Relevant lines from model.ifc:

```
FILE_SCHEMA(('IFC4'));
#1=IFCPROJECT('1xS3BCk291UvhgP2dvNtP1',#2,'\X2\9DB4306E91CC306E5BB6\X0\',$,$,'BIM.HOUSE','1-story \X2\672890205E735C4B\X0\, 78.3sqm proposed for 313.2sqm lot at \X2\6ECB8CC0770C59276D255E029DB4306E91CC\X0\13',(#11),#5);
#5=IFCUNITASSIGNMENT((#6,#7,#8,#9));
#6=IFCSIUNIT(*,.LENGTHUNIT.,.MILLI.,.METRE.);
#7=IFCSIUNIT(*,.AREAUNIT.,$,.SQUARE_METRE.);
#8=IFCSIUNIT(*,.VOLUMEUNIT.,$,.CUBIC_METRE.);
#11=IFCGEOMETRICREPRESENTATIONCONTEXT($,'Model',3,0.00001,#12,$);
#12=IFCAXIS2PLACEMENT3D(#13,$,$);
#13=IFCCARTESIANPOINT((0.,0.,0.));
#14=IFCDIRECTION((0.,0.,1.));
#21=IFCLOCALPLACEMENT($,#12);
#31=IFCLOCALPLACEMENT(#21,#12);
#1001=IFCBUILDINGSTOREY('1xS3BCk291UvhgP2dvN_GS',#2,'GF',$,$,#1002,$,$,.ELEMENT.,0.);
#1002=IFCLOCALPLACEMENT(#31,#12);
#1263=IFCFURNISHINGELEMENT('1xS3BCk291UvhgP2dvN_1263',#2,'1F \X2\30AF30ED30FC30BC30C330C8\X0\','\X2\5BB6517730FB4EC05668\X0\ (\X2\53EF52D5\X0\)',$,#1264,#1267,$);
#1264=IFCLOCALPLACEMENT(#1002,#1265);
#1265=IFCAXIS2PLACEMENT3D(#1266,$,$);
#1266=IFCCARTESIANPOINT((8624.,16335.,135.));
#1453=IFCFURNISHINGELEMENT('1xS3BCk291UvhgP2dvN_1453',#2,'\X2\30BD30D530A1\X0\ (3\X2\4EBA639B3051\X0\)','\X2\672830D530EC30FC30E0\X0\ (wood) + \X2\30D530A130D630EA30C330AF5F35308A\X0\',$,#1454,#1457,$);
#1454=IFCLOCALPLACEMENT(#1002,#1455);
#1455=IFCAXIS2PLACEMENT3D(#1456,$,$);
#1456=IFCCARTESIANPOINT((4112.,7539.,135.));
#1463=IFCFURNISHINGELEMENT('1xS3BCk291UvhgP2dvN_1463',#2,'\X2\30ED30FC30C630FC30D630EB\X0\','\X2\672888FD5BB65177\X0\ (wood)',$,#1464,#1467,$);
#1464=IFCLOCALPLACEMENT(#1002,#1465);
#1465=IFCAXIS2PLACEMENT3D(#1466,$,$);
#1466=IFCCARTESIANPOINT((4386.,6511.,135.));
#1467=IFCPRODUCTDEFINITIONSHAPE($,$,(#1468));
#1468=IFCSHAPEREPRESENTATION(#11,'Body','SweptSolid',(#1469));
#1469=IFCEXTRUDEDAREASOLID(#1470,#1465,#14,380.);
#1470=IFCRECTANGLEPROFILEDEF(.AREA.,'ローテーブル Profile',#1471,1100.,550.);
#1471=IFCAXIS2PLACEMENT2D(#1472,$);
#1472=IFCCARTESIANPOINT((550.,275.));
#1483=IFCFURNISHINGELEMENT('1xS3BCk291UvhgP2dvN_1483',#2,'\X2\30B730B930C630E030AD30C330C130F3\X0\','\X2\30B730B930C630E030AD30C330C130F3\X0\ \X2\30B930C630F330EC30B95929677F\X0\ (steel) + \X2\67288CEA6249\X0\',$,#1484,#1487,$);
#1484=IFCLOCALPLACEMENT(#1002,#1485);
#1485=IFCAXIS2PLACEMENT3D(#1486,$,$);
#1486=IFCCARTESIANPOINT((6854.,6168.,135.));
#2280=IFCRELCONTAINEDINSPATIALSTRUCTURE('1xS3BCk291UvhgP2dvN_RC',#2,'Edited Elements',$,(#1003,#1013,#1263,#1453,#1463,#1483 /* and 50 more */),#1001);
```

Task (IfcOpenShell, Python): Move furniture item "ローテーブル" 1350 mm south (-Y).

```python
import ifcopenshell
import ifcopenshell.api.geometry
import ifcopenshell.util.placement

model = ifcopenshell.open("model.ifc")

item = model.by_guid("1xS3BCk291UvhgP2dvN_1463")
matrix = ifcopenshell.util.placement.get_local_placement(item.ObjectPlacement)
matrix[1, 3] -= 1350.0
ifcopenshell.api.geometry.edit_object_placement(model, product=item, matrix=matrix, is_si=False)

print(ifcopenshell.util.placement.get_local_placement(item.ObjectPlacement).round(3) + 0.0)

model.write("model_edited.ifc")
```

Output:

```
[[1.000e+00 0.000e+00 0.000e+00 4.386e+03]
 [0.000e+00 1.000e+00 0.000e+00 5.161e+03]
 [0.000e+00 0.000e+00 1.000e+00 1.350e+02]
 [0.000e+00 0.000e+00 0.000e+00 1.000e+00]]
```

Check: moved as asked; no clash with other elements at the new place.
